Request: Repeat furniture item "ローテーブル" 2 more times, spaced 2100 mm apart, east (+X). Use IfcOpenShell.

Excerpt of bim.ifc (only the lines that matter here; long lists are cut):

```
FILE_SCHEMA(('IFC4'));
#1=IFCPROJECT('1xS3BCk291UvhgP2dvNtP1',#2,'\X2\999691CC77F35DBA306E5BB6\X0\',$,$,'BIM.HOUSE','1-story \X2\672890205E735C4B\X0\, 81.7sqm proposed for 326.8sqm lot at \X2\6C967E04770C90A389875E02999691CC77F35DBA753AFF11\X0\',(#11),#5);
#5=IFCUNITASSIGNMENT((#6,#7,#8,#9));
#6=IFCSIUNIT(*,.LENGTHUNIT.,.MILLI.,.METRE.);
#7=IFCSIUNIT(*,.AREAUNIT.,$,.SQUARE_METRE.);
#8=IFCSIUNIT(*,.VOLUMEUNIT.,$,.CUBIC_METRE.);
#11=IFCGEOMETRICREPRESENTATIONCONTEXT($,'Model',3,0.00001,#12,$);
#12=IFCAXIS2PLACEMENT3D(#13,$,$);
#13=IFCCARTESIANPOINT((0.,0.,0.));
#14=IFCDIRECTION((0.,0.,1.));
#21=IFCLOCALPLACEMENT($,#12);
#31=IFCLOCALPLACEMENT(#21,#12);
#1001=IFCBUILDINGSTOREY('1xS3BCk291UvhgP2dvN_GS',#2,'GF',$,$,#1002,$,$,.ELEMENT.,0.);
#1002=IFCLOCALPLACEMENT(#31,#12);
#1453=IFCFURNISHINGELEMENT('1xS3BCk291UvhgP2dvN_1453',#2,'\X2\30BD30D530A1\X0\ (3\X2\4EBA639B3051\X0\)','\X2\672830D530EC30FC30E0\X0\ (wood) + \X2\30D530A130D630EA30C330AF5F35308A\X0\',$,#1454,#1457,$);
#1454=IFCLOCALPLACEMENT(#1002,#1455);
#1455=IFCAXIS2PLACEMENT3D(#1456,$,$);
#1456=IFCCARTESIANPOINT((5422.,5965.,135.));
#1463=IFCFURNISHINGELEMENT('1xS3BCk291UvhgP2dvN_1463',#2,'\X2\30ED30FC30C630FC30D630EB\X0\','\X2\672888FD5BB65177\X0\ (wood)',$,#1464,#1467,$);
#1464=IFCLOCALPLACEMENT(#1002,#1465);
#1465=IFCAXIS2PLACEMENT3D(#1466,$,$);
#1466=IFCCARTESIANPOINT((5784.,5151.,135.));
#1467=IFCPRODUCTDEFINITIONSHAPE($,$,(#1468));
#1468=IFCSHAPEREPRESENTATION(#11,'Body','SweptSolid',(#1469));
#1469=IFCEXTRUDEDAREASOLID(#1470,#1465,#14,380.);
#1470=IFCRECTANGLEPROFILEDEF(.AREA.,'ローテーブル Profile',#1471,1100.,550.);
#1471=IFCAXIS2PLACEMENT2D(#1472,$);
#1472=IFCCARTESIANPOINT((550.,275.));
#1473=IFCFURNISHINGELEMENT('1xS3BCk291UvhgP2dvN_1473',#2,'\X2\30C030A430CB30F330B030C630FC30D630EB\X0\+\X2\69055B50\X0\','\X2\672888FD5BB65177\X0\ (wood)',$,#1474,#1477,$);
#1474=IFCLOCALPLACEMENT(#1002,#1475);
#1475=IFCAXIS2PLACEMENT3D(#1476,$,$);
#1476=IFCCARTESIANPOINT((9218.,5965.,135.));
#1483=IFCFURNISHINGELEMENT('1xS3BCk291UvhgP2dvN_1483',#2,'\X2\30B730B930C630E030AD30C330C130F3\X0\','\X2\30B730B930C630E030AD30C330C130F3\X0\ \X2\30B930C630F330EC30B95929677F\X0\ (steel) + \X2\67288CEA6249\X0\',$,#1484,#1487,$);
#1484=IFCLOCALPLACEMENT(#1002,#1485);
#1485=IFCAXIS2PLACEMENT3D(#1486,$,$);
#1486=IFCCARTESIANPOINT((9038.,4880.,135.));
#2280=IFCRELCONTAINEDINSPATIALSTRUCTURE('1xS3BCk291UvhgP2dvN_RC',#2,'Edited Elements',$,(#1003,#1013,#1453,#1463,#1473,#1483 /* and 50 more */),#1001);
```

```python
import numpy as np
import ifcopenshell
import ifcopenshell.api.geometry
import ifcopenshell.api.root
import ifcopenshell.util.element
import ifcopenshell.util.placement

model = ifcopenshell.open("bim.ifc")


def reuse_history(source, copy):
    """copy_class also copies each property set's owner history, people and application; keep the originals."""
    for rel in copy.IsDefinedBy:
        if rel.is_a("IfcRelDefinesByProperties") and (history := rel.RelatingPropertyDefinition.OwnerHistory):
            rel.RelatingPropertyDefinition.OwnerHistory = source.OwnerHistory
            ifcopenshell.util.element.remove_deep2(model, history)


source = model.by_id(1463)
base = ifcopenshell.util.placement.get_local_placement(source.ObjectPlacement)
step = np.array([1.0, 0.0, 0.0]) * 2100.0

for i in range(1, 3):
    copy = ifcopenshell.api.root.copy_class(model, product=source)
    copy.Representation = ifcopenshell.util.element.copy_deep(
        model, source.Representation, exclude=["IfcGeometricRepresentationContext", "IfcRepresentationMap"]
    )
    reuse_history(source, copy)
    matrix = base.copy()
    matrix[:3, 3] += i * step
    print("added at", matrix[:3, 3].round(3) + 0.0)
    ifcopenshell.api.geometry.edit_object_placement(model, product=copy, matrix=matrix, is_si=False)

model.write("bim-out.ifc")
```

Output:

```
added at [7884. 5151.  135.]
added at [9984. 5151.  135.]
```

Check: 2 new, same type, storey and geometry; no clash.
